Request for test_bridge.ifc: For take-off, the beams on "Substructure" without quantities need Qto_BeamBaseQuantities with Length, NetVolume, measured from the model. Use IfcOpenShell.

First a look at what the model holds.

```python
import ifcopenshell
import ifcopenshell.util.element
import ifcopenshell.util.unit

model = ifcopenshell.open("test_bridge.ifc")
print(model.schema)
for unit_type in ("LENGTHUNIT", "AREAUNIT", "VOLUMEUNIT"):
    print(unit_type, ifcopenshell.util.unit.calculate_unit_scale(model, unit_type))
storey = next(s for s in model.by_type("IfcBuildingStorey") if s.Name == "Substructure")
beams = [e for e in ifcopenshell.util.element.get_decomposition(storey) if e.is_a("IfcBeam")]
for e in sorted(beams, key=lambda e: e.id()):
    print(e.id(), e.is_a(), e.Name, list(ifcopenshell.util.element.get_psets(e, qtos_only=True)), sep=" | ")
```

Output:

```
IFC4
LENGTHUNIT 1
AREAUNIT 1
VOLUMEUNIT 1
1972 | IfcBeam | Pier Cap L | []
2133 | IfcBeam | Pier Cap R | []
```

```python
import ifcopenshell
import ifcopenshell.api.pset
import ifcopenshell.geom
import ifcopenshell.util.element
import ifcopenshell.util.shape
import ifcopenshell.util.unit

model = ifcopenshell.open("test_bridge.ifc")
unit_scale = ifcopenshell.util.unit.calculate_unit_scale(model)
volume_scale = ifcopenshell.util.unit.calculate_unit_scale(model, "VOLUMEUNIT")
settings = ifcopenshell.geom.settings()

storey = next(s for s in model.by_type("IfcBuildingStorey") if s.Name == "Substructure")
beams = [e for e in ifcopenshell.util.element.get_decomposition(storey) if e.is_a("IfcBeam")]

for e in sorted(beams, key=lambda e: e.id()):
    if ifcopenshell.util.element.get_psets(e, qtos_only=True, should_inherit=False):
        continue
    # Geometry comes back in metres, in the element's own axes.
    shape = ifcopenshell.geom.create_shape(settings, e)
    values = {
        "Length": ifcopenshell.util.shape.get_max_xyz(shape.geometry) / unit_scale,
        "NetVolume": ifcopenshell.util.shape.get_volume(shape.geometry) / volume_scale,
    }
    qto = ifcopenshell.api.pset.add_qto(model, product=e, name="Qto_BeamBaseQuantities")
    ifcopenshell.api.pset.edit_qto(model, qto=qto, properties=values)
    print(e.id(), {k: round(v, 3) for k, v in values.items()})

model.write("test_bridge-out.ifc")
```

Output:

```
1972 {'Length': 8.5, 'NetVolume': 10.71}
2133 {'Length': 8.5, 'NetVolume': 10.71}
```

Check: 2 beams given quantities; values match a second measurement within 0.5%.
